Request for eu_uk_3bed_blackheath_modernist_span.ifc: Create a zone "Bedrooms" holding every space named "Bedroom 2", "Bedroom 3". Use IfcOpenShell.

First a look at what the model holds.

```python
import ifcopenshell

model = ifcopenshell.open("eu_uk_3bed_blackheath_modernist_span.ifc")
print(model.schema)
seen = {}
for space in model.by_type("IfcSpace"):
    seen[space.LongName] = seen.get(space.LongName, 0) + 1
for name, count in sorted(seen.items(), key=str):
    print(count, "x", name)
print("zones:", [z.Name for z in model.by_type("IfcZone")][:20])
```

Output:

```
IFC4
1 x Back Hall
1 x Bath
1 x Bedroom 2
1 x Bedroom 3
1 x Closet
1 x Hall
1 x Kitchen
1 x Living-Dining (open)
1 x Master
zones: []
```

```python
import ifcopenshell
import ifcopenshell.api.group
import ifcopenshell.api.root

model = ifcopenshell.open("eu_uk_3bed_blackheath_modernist_span.ifc")

names = {"Bedroom 2", "Bedroom 3"}
spaces = [s for s in model.by_type("IfcSpace") if s.LongName in names]

zone = ifcopenshell.api.root.create_entity(model, ifc_class="IfcZone", name="Bedrooms")
ifcopenshell.api.group.assign_group(model, products=spaces, group=zone)
print(len(spaces), "spaces in", zone.Name)

model.write("eu_uk_3bed_blackheath_modernist_span_rev.ifc")
```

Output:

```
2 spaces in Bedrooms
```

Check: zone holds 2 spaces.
